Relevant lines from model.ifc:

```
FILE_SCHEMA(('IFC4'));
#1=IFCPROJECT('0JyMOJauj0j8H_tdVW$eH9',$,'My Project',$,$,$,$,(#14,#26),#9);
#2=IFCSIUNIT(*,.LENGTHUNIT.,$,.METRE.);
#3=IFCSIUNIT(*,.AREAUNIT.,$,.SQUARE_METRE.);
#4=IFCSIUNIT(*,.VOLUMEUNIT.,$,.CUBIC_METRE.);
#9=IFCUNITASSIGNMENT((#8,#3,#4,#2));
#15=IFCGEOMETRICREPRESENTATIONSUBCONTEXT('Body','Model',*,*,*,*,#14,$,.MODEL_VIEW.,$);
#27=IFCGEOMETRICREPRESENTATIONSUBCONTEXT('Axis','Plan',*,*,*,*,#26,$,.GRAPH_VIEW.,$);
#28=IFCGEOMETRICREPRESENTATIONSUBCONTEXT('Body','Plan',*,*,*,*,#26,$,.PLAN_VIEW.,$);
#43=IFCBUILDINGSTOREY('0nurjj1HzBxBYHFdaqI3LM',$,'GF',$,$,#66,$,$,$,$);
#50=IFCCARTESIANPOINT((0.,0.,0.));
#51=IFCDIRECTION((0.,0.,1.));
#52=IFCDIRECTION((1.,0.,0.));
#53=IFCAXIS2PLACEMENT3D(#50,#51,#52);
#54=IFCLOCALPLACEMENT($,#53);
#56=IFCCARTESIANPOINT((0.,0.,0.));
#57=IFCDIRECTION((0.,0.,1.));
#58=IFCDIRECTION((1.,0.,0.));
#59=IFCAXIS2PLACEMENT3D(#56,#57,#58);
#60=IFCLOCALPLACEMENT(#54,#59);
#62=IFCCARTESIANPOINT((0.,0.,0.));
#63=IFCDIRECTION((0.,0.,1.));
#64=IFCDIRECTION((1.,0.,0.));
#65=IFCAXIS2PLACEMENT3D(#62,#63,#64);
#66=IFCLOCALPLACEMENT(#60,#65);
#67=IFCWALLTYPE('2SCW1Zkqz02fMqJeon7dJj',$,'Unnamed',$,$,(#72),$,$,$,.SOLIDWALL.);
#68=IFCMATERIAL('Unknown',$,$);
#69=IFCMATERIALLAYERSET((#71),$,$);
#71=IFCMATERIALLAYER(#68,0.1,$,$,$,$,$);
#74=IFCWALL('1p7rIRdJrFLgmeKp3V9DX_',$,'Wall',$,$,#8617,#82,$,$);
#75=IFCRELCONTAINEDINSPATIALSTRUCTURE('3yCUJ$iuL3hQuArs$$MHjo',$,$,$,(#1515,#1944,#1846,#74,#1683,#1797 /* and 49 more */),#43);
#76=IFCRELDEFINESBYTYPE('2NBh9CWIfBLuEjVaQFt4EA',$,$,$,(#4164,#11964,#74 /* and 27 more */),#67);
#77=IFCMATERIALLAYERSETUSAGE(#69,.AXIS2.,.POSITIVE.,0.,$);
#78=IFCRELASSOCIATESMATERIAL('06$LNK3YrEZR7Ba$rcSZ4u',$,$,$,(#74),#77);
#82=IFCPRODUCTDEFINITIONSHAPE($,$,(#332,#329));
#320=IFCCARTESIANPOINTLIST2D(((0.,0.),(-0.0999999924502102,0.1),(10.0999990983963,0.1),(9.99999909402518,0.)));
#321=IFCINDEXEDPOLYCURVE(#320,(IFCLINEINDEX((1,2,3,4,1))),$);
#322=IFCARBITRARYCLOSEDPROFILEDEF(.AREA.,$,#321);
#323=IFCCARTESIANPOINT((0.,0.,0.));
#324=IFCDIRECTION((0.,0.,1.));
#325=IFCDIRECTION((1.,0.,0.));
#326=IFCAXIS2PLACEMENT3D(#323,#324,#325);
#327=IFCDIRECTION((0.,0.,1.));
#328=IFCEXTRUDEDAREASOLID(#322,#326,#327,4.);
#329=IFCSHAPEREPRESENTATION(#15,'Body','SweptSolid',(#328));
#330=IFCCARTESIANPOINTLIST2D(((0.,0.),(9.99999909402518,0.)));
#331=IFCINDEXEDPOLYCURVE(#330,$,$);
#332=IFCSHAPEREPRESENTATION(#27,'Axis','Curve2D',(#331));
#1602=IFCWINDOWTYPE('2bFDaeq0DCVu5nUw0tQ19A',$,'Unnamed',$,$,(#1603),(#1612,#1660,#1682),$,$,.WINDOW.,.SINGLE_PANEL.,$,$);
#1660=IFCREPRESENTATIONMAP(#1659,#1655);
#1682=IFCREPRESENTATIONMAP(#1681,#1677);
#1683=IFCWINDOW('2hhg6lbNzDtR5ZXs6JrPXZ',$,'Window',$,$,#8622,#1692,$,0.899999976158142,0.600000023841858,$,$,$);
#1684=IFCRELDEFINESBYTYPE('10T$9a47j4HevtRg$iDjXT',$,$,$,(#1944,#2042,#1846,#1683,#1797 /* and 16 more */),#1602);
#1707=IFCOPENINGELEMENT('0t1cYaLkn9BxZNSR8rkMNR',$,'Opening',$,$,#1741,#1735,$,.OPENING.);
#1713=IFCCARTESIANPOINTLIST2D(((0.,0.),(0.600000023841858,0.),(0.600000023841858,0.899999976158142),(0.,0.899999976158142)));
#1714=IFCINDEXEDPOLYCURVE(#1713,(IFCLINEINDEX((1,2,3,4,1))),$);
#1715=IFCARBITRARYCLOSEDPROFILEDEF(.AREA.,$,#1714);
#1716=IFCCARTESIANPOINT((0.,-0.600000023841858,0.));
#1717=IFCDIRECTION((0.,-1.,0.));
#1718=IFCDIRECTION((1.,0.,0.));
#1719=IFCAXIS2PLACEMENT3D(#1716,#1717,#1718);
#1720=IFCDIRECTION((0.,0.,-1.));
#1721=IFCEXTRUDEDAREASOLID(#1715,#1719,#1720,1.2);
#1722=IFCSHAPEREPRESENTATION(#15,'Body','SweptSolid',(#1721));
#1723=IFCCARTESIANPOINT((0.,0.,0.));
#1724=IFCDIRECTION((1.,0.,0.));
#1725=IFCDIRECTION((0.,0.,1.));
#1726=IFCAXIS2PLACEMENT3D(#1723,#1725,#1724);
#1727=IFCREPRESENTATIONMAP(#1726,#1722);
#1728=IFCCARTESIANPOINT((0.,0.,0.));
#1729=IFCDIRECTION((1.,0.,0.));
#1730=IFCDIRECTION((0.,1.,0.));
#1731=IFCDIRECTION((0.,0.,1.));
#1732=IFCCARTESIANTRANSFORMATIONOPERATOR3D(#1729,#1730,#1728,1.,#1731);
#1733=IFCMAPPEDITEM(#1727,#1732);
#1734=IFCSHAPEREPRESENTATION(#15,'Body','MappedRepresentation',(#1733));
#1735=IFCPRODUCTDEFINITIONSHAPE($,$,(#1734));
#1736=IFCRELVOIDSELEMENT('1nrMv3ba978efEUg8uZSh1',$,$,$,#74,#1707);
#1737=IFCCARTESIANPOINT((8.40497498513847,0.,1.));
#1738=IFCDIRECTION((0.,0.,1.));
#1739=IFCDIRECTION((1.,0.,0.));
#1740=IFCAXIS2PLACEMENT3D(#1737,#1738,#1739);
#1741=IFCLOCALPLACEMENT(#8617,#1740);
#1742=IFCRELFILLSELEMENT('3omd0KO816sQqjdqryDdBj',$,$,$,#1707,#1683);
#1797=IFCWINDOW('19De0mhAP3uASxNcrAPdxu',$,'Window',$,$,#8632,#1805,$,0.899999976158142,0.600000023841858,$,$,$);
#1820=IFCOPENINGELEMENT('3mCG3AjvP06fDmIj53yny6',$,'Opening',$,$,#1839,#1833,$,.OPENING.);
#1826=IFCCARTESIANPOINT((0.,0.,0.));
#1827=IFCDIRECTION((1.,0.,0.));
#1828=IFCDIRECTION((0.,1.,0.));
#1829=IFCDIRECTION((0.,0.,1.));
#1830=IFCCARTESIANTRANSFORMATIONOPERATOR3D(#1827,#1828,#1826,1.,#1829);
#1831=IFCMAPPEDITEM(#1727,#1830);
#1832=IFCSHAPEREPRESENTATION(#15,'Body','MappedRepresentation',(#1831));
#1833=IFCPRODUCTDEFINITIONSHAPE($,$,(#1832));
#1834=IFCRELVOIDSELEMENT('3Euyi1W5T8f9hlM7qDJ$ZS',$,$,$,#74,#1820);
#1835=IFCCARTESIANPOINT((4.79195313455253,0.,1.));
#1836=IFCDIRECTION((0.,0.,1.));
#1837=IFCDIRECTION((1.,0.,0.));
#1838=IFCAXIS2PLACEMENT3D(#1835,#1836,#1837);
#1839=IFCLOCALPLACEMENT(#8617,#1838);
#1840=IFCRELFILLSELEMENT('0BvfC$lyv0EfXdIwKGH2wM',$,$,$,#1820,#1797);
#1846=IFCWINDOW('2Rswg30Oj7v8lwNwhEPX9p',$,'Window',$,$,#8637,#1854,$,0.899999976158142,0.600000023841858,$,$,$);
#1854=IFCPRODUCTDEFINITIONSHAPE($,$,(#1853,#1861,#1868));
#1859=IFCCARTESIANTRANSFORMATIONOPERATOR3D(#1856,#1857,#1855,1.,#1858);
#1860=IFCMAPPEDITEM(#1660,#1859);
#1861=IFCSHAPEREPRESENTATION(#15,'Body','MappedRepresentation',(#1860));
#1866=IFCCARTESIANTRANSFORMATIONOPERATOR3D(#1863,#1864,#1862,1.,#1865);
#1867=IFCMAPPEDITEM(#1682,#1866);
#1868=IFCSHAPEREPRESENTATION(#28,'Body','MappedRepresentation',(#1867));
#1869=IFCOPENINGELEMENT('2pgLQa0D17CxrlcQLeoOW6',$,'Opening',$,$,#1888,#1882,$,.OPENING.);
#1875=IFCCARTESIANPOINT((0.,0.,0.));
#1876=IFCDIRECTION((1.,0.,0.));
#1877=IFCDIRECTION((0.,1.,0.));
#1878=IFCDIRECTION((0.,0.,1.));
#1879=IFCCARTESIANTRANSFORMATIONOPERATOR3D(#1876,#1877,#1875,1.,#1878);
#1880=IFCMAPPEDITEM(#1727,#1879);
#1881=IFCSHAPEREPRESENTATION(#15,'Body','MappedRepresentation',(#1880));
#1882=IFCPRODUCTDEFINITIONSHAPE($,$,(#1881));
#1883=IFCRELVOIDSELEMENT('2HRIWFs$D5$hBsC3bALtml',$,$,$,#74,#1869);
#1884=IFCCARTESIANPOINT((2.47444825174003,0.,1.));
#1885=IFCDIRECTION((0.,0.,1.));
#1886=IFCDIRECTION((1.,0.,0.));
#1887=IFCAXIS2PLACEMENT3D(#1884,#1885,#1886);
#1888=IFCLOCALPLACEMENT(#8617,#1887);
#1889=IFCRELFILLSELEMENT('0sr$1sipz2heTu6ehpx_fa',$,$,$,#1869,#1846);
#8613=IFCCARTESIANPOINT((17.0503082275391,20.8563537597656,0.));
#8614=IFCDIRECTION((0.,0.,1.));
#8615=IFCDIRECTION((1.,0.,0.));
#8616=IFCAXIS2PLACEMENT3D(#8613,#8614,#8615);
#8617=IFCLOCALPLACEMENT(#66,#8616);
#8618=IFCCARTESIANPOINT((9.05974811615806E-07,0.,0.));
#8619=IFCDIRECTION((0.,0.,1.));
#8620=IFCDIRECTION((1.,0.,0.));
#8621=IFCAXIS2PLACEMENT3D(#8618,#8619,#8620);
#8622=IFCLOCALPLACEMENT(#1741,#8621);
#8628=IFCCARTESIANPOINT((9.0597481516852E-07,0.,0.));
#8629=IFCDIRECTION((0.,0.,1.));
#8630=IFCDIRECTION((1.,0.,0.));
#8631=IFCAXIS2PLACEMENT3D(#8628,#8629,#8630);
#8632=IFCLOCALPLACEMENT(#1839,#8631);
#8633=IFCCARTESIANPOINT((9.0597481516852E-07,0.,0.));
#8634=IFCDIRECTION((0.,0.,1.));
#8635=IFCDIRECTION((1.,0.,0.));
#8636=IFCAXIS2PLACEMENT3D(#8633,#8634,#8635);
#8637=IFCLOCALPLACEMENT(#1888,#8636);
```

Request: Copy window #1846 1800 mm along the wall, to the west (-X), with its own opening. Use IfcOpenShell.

```python
import ifcopenshell
import ifcopenshell.api.feature
import ifcopenshell.api.geometry
import ifcopenshell.api.root
import ifcopenshell.geom
import ifcopenshell.util.element
import ifcopenshell.util.placement
import ifcopenshell.util.shape
import ifcopenshell.util.unit

model = ifcopenshell.open("model.ifc")
unit_scale = ifcopenshell.util.unit.calculate_unit_scale(model)
settings = ifcopenshell.geom.settings()


def volume(element):
    """Net volume in cubic metres, openings subtracted."""
    shape = ifcopenshell.geom.create_shape(settings, element)
    return ifcopenshell.util.shape.get_volume(shape.geometry)


window = model.by_guid("2Rswg30Oj7v8lwNwhEPX9p")
opening = window.FillsVoids[0].RelatingOpeningElement
wall = opening.VoidsElements[0].RelatingBuildingElement
before = volume(wall)
shift = ifcopenshell.util.placement.get_local_placement(wall.ObjectPlacement)[:3, 0] * -1.8 / unit_scale

# copy_class copies the void relationship, type, container and properties, but no geometry.
new_opening = ifcopenshell.api.root.copy_class(model, product=opening)
new_opening.Representation = ifcopenshell.util.element.copy_deep(
    model, opening.Representation, exclude=["IfcGeometricRepresentationContext", "IfcRepresentationMap"]
)
new_window = ifcopenshell.api.root.copy_class(model, product=window)
new_window.Representation = ifcopenshell.util.element.copy_deep(
    model, window.Representation, exclude=["IfcGeometricRepresentationContext", "IfcRepresentationMap"]
)
ifcopenshell.api.feature.add_filling(model, opening=new_opening, element=new_window)

for old, new in ((opening, new_opening), (window, new_window)):
    matrix = ifcopenshell.util.placement.get_local_placement(old.ObjectPlacement)
    matrix[:3, 3] += shift
    ifcopenshell.api.geometry.edit_object_placement(model, product=new, matrix=matrix, is_si=False)

after = volume(wall)

print(f"wall volume {before:.3f} -> {after:.3f} m3")

model.write("model_edited.ifc")
```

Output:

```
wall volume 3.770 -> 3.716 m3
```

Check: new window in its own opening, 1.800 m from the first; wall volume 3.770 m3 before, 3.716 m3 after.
